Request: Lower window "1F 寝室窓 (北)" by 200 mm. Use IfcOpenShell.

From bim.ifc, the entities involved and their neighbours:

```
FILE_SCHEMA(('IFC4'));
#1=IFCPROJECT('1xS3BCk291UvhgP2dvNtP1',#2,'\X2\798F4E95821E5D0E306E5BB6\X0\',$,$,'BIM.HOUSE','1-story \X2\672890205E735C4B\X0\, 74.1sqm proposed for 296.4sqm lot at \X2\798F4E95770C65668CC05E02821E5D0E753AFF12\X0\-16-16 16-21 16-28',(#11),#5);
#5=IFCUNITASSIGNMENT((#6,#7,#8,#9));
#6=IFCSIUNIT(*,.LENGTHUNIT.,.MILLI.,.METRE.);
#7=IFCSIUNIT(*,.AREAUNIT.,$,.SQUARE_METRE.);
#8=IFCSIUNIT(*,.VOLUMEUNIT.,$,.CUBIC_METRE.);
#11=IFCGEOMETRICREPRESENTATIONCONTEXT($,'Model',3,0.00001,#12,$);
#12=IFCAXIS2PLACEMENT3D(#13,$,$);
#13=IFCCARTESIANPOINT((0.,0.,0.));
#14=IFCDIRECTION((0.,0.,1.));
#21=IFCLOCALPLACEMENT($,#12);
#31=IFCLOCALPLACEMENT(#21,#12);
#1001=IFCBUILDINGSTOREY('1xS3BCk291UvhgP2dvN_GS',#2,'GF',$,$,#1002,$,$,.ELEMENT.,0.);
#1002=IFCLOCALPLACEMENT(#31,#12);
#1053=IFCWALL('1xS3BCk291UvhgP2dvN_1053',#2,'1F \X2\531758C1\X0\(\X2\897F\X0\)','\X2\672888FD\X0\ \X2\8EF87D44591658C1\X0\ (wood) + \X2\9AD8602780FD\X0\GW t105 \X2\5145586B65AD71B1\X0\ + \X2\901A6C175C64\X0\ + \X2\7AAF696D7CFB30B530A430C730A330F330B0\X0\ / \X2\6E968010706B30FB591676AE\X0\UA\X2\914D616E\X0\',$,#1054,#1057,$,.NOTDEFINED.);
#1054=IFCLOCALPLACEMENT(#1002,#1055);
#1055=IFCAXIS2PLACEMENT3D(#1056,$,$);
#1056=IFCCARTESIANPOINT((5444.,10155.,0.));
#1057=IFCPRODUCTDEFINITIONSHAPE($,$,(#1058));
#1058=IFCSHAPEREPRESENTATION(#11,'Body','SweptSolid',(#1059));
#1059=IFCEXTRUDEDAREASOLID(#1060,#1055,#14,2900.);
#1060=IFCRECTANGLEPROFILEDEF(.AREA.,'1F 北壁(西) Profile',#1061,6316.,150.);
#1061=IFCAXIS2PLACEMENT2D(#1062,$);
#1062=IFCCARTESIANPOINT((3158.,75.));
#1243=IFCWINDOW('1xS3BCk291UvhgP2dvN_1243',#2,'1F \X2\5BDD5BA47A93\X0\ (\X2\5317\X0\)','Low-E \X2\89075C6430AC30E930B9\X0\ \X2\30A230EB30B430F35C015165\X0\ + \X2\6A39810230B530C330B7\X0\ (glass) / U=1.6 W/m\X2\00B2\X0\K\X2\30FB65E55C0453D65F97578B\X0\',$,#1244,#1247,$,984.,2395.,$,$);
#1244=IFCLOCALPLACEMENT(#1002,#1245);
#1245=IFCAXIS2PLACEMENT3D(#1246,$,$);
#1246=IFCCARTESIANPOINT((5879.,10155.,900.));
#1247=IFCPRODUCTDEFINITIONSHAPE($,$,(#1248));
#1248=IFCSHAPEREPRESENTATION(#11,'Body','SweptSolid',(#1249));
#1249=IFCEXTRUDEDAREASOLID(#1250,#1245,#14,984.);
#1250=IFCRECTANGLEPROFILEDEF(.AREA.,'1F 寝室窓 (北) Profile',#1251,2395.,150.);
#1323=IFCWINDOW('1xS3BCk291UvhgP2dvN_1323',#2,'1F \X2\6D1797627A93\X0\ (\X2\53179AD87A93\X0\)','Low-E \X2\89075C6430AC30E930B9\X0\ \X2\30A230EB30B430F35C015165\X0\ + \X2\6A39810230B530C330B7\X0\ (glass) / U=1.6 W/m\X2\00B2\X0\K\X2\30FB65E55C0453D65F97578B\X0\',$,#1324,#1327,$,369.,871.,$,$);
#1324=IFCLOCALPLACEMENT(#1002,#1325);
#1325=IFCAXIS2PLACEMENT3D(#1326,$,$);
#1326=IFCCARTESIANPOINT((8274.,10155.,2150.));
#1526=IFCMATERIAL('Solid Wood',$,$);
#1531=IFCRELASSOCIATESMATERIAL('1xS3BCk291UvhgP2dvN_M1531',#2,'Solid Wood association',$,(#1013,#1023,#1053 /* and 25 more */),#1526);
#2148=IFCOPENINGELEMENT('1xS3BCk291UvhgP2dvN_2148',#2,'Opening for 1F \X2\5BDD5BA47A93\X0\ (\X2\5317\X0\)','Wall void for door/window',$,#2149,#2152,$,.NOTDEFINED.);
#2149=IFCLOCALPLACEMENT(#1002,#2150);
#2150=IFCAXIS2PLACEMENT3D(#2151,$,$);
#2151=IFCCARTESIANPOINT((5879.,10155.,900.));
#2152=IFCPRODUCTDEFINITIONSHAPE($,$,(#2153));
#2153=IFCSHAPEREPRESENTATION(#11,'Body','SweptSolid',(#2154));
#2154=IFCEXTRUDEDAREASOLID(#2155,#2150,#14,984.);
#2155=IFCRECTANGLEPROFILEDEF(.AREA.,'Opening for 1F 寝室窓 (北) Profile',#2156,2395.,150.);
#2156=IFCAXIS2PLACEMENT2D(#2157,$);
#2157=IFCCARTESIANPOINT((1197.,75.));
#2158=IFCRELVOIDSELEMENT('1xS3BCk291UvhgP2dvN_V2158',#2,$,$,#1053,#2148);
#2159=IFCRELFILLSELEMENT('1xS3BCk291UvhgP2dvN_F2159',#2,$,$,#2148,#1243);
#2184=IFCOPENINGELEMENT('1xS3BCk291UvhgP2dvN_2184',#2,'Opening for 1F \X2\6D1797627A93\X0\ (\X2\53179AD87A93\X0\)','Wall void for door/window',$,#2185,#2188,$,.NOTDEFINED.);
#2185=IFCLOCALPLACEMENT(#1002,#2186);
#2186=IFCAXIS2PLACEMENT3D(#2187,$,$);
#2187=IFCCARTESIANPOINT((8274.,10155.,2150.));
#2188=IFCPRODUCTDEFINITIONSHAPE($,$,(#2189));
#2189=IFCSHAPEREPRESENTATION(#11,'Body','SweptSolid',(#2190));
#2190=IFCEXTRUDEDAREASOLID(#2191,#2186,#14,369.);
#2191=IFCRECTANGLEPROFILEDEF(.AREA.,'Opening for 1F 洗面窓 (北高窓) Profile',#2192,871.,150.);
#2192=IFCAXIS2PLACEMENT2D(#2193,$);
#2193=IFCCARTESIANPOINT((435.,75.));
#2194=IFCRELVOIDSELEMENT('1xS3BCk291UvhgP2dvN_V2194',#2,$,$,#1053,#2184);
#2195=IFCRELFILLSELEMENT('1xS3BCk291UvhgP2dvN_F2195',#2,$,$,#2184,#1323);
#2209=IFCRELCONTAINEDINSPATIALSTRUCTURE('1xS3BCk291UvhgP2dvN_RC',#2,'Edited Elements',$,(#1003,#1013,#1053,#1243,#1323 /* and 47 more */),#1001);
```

```python
import numpy as np
import ifcopenshell
import ifcopenshell.api.geometry
import ifcopenshell.util.placement
import ifcopenshell.util.unit

model = ifcopenshell.open("bim.ifc")
unit_scale = ifcopenshell.util.unit.calculate_unit_scale(model)

window = model.by_guid("1xS3BCk291UvhgP2dvN_1243")
opening = window.FillsVoids[0].RelatingOpeningElement
dz = -200.0

shift = np.array([0.0, 0.0, dz])
# The window is not placed relative to its opening, so move both.
for product in (opening, window):
    matrix = ifcopenshell.util.placement.get_local_placement(product.ObjectPlacement)
    matrix[:3, 3] += shift
    ifcopenshell.api.geometry.edit_object_placement(model, product=product, matrix=matrix, is_si=False)

print(f"moved by {dz * unit_scale:+.3f} m")

model.write("bim_rev.ifc")
```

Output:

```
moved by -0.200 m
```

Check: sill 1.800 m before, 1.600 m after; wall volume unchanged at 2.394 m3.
